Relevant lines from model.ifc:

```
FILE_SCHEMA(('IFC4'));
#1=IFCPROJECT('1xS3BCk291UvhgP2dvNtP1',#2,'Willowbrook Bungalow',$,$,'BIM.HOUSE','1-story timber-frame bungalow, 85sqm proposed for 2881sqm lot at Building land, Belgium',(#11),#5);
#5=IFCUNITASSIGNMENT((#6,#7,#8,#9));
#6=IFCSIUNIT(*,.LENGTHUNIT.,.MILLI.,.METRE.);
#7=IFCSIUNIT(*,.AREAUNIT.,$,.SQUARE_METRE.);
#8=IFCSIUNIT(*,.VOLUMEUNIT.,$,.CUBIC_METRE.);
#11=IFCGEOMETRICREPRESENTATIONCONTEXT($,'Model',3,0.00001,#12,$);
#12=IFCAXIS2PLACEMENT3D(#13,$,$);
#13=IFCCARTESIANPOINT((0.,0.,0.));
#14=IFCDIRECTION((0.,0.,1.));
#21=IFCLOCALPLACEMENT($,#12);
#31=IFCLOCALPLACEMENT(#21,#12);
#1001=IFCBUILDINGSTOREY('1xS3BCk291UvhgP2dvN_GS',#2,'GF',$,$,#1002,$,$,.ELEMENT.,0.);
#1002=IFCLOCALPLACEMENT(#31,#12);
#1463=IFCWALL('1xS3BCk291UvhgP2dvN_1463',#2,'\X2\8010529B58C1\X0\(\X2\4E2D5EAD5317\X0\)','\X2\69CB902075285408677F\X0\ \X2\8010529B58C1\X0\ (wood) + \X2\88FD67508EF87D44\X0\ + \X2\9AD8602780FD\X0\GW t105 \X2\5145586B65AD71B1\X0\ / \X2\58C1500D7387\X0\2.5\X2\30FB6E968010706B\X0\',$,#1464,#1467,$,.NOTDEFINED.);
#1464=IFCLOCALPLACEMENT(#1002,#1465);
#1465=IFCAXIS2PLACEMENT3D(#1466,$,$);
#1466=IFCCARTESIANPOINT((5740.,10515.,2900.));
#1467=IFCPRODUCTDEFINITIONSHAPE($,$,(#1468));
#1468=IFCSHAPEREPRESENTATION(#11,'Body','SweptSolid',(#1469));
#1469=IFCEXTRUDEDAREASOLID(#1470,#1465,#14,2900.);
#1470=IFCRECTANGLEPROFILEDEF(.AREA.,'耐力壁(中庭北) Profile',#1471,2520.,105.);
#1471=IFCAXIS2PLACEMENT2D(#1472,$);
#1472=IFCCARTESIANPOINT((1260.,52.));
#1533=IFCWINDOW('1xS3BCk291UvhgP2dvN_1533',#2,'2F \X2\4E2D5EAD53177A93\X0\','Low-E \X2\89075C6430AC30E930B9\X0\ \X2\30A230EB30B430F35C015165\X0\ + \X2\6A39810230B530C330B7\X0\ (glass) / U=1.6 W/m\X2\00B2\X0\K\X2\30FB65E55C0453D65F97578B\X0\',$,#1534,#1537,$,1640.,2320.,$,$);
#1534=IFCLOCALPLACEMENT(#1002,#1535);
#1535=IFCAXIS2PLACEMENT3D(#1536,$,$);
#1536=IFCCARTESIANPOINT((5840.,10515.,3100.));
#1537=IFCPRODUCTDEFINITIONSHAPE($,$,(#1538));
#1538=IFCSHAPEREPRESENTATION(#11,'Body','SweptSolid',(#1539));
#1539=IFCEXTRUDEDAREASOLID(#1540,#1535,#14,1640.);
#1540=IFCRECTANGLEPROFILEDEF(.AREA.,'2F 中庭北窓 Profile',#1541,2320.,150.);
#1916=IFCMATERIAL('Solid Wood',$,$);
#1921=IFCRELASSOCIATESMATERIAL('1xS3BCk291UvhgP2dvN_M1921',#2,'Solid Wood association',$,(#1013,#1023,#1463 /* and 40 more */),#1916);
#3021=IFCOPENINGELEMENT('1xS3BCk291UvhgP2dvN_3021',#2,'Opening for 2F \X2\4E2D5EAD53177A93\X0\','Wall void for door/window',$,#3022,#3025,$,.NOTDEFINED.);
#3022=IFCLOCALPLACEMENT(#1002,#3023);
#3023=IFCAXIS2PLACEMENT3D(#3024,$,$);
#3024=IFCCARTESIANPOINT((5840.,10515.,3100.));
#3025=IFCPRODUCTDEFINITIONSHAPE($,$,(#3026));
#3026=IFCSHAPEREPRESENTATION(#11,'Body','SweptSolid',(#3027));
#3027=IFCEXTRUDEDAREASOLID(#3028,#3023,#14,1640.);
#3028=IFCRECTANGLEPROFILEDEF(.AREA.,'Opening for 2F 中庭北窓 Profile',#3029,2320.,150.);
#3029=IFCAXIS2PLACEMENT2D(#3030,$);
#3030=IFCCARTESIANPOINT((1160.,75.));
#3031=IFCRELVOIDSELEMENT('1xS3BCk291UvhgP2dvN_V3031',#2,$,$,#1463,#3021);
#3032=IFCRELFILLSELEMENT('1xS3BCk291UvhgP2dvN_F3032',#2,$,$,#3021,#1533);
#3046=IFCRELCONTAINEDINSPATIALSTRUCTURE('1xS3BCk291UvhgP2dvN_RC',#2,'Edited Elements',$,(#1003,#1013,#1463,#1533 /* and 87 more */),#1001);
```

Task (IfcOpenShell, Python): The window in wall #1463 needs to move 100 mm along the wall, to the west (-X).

```python
import ifcopenshell
import ifcopenshell.api.geometry
import ifcopenshell.util.placement
import ifcopenshell.util.unit

model = ifcopenshell.open("model.ifc")
unit_scale = ifcopenshell.util.unit.calculate_unit_scale(model)

window = model.by_guid("1xS3BCk291UvhgP2dvN_1533")
opening = window.FillsVoids[0].RelatingOpeningElement
wall = opening.VoidsElements[0].RelatingBuildingElement

wall_matrix = ifcopenshell.util.placement.get_local_placement(wall.ObjectPlacement)
shift = wall_matrix[:3, 0] * -0.1 / unit_scale
before = ifcopenshell.util.placement.get_local_placement(window.ObjectPlacement)[:3, 3].copy()

# The window is not placed relative to its opening, so move both.
for product in (opening, window):
    matrix = ifcopenshell.util.placement.get_local_placement(product.ObjectPlacement)
    matrix[:3, 3] += shift
    ifcopenshell.api.geometry.edit_object_placement(model, product=product, matrix=matrix, is_si=False)

after = ifcopenshell.util.placement.get_local_placement(window.ObjectPlacement)[:3, 3]
print("window moved by", (after - before).round(3) + 0.0)

model.write("model_rev.ifc")
```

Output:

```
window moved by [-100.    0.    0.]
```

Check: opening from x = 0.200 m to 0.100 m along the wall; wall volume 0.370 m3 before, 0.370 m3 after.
